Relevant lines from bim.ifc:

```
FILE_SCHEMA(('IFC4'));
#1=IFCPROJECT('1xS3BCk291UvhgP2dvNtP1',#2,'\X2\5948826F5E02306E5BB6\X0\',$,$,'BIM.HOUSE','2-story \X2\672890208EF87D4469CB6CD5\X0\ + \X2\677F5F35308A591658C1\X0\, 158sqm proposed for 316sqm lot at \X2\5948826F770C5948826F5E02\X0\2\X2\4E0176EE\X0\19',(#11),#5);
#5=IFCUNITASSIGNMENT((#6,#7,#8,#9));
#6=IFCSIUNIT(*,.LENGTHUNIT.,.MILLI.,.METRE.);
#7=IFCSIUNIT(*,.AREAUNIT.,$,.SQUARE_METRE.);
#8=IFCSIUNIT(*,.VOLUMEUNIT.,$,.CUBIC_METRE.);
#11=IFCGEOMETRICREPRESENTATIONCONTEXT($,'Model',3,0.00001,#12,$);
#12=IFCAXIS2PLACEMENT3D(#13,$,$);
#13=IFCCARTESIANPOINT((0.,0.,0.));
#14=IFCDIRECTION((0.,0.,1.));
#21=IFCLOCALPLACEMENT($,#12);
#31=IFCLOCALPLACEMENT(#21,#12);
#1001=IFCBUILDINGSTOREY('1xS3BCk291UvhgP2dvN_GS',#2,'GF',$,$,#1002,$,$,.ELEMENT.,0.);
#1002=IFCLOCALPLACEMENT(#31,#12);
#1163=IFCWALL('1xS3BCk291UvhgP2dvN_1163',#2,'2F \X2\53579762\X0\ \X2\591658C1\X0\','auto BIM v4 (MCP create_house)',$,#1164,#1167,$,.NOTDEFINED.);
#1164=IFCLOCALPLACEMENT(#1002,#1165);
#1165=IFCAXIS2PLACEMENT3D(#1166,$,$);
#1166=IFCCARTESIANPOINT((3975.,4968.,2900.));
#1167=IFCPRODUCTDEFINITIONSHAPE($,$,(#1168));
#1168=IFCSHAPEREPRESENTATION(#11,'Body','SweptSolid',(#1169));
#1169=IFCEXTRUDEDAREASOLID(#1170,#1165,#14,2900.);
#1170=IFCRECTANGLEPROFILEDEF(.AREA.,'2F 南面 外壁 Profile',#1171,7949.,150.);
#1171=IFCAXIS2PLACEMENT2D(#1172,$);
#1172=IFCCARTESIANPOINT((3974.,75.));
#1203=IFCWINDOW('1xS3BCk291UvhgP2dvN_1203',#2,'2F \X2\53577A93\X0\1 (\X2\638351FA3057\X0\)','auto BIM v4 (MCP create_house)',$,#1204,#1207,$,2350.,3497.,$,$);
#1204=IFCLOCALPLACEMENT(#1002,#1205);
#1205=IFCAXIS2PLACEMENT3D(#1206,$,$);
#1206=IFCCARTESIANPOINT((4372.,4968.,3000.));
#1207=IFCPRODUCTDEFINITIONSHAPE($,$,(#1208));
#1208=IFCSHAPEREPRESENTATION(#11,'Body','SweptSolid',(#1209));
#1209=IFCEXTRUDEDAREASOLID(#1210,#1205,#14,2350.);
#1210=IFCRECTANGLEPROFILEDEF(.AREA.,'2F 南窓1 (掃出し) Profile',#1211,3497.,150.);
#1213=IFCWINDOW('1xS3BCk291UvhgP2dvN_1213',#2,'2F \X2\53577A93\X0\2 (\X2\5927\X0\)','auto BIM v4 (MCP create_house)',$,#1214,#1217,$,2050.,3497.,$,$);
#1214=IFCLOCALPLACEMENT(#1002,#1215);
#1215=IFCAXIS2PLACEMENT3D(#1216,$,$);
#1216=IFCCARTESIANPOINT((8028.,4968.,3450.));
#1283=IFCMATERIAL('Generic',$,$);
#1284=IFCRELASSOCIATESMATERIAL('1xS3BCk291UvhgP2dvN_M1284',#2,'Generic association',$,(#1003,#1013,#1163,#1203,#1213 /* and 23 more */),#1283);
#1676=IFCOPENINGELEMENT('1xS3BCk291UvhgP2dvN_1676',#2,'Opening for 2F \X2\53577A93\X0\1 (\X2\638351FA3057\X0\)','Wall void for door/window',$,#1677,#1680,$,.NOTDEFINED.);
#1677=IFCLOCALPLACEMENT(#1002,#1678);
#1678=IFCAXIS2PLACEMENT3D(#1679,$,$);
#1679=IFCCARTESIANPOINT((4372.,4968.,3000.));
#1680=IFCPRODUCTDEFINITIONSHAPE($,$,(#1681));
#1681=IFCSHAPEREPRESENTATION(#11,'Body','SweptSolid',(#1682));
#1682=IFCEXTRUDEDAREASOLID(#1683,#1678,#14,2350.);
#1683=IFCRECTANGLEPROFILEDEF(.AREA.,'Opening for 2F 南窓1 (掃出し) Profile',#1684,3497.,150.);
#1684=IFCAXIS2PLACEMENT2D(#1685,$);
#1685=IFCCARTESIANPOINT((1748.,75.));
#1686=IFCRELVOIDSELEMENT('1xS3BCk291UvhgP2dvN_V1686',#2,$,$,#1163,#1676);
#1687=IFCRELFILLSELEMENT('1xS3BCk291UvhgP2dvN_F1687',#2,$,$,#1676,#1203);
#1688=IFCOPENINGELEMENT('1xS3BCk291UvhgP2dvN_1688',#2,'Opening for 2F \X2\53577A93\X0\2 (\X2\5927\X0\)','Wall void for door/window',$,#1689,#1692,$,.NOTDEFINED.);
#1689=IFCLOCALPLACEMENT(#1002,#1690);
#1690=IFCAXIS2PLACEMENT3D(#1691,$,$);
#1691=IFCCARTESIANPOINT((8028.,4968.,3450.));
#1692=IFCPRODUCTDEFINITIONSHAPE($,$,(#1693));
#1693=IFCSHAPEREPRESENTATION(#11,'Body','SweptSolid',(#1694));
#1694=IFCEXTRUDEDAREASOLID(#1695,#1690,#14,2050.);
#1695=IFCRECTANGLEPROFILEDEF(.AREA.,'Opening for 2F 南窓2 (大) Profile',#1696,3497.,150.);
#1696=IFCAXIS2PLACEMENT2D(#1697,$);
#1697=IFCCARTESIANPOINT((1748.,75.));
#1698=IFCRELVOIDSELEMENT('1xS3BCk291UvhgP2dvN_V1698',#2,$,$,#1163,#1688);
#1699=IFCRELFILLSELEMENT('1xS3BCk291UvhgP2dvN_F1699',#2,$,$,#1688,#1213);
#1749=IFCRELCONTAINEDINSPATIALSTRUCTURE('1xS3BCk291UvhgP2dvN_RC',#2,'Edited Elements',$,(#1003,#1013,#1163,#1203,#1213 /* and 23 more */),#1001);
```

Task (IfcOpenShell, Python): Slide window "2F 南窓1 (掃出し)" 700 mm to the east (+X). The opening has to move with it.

```python
import ifcopenshell
import ifcopenshell.api.geometry
import ifcopenshell.util.placement

model = ifcopenshell.open("bim.ifc")

window = model.by_guid("1xS3BCk291UvhgP2dvN_1203")
opening = window.FillsVoids[0].RelatingOpeningElement
wall = opening.VoidsElements[0].RelatingBuildingElement

wall_matrix = ifcopenshell.util.placement.get_local_placement(wall.ObjectPlacement)
shift = wall_matrix[:3, 0] * 700.0
before = ifcopenshell.util.placement.get_local_placement(window.ObjectPlacement)[:3, 3].copy()

# The window is not placed relative to its opening, so move both.
for product in (opening, window):
    matrix = ifcopenshell.util.placement.get_local_placement(product.ObjectPlacement)
    matrix[:3, 3] += shift
    ifcopenshell.api.geometry.edit_object_placement(model, product=product, matrix=matrix, is_si=False)

after = ifcopenshell.util.placement.get_local_placement(window.ObjectPlacement)[:3, 3]
print("window moved by", (after - before).round(3) + 0.0)

model.write("bim-out.ifc")
```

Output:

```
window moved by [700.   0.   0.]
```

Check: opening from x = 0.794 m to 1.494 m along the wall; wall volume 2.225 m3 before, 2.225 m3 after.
